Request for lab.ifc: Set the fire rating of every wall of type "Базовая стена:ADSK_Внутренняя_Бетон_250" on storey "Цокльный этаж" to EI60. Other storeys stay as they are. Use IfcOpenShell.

First a look at what the model holds.

```python
import ifcopenshell
import ifcopenshell.util.element

model = ifcopenshell.open("lab.ifc")
print(model.schema)
storey = next(s for s in model.by_type("IfcBuildingStorey") if s.Name == "Цокльный этаж")
walls = [e for e in ifcopenshell.util.element.get_decomposition(storey) if e.is_a("IfcWall")]
seen = {}
for e in walls:
    element_type = ifcopenshell.util.element.get_type(e)
    key = (element_type.Name if element_type != e and element_type else None, ifcopenshell.util.element.get_pset(e, "Pset_WallCommon", "FireRating"))
    seen[key] = seen.get(key, 0) + 1
for (name, value), count in sorted(seen.items(), key=str):
    print(count, "x", name, "|", value)
```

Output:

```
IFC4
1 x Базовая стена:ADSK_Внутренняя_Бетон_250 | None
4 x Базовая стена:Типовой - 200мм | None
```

```python
import ifcopenshell
import ifcopenshell.api.pset
import ifcopenshell.util.element

model = ifcopenshell.open("lab.ifc")

storey = next(s for s in model.by_type("IfcBuildingStorey") if s.Name == "Цокльный этаж")
walls = [e for e in ifcopenshell.util.element.get_decomposition(storey) if e.is_a("IfcWall")]

count = 0
for e in walls:
    element_type = ifcopenshell.util.element.get_type(e)
    if element_type in (None, e) or element_type.Name != "Базовая стена:ADSK_Внутренняя_Бетон_250":
        continue
    # add_pset returns the element's existing set when there is one.
    pset = ifcopenshell.api.pset.add_pset(model, product=e, name="Pset_WallCommon")
    ifcopenshell.api.pset.edit_pset(model, pset=pset, properties={"FireRating": "EI60"})
    count += 1

print(count, "walls updated")

model.write("lab_v2.ifc")
```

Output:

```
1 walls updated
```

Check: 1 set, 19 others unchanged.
